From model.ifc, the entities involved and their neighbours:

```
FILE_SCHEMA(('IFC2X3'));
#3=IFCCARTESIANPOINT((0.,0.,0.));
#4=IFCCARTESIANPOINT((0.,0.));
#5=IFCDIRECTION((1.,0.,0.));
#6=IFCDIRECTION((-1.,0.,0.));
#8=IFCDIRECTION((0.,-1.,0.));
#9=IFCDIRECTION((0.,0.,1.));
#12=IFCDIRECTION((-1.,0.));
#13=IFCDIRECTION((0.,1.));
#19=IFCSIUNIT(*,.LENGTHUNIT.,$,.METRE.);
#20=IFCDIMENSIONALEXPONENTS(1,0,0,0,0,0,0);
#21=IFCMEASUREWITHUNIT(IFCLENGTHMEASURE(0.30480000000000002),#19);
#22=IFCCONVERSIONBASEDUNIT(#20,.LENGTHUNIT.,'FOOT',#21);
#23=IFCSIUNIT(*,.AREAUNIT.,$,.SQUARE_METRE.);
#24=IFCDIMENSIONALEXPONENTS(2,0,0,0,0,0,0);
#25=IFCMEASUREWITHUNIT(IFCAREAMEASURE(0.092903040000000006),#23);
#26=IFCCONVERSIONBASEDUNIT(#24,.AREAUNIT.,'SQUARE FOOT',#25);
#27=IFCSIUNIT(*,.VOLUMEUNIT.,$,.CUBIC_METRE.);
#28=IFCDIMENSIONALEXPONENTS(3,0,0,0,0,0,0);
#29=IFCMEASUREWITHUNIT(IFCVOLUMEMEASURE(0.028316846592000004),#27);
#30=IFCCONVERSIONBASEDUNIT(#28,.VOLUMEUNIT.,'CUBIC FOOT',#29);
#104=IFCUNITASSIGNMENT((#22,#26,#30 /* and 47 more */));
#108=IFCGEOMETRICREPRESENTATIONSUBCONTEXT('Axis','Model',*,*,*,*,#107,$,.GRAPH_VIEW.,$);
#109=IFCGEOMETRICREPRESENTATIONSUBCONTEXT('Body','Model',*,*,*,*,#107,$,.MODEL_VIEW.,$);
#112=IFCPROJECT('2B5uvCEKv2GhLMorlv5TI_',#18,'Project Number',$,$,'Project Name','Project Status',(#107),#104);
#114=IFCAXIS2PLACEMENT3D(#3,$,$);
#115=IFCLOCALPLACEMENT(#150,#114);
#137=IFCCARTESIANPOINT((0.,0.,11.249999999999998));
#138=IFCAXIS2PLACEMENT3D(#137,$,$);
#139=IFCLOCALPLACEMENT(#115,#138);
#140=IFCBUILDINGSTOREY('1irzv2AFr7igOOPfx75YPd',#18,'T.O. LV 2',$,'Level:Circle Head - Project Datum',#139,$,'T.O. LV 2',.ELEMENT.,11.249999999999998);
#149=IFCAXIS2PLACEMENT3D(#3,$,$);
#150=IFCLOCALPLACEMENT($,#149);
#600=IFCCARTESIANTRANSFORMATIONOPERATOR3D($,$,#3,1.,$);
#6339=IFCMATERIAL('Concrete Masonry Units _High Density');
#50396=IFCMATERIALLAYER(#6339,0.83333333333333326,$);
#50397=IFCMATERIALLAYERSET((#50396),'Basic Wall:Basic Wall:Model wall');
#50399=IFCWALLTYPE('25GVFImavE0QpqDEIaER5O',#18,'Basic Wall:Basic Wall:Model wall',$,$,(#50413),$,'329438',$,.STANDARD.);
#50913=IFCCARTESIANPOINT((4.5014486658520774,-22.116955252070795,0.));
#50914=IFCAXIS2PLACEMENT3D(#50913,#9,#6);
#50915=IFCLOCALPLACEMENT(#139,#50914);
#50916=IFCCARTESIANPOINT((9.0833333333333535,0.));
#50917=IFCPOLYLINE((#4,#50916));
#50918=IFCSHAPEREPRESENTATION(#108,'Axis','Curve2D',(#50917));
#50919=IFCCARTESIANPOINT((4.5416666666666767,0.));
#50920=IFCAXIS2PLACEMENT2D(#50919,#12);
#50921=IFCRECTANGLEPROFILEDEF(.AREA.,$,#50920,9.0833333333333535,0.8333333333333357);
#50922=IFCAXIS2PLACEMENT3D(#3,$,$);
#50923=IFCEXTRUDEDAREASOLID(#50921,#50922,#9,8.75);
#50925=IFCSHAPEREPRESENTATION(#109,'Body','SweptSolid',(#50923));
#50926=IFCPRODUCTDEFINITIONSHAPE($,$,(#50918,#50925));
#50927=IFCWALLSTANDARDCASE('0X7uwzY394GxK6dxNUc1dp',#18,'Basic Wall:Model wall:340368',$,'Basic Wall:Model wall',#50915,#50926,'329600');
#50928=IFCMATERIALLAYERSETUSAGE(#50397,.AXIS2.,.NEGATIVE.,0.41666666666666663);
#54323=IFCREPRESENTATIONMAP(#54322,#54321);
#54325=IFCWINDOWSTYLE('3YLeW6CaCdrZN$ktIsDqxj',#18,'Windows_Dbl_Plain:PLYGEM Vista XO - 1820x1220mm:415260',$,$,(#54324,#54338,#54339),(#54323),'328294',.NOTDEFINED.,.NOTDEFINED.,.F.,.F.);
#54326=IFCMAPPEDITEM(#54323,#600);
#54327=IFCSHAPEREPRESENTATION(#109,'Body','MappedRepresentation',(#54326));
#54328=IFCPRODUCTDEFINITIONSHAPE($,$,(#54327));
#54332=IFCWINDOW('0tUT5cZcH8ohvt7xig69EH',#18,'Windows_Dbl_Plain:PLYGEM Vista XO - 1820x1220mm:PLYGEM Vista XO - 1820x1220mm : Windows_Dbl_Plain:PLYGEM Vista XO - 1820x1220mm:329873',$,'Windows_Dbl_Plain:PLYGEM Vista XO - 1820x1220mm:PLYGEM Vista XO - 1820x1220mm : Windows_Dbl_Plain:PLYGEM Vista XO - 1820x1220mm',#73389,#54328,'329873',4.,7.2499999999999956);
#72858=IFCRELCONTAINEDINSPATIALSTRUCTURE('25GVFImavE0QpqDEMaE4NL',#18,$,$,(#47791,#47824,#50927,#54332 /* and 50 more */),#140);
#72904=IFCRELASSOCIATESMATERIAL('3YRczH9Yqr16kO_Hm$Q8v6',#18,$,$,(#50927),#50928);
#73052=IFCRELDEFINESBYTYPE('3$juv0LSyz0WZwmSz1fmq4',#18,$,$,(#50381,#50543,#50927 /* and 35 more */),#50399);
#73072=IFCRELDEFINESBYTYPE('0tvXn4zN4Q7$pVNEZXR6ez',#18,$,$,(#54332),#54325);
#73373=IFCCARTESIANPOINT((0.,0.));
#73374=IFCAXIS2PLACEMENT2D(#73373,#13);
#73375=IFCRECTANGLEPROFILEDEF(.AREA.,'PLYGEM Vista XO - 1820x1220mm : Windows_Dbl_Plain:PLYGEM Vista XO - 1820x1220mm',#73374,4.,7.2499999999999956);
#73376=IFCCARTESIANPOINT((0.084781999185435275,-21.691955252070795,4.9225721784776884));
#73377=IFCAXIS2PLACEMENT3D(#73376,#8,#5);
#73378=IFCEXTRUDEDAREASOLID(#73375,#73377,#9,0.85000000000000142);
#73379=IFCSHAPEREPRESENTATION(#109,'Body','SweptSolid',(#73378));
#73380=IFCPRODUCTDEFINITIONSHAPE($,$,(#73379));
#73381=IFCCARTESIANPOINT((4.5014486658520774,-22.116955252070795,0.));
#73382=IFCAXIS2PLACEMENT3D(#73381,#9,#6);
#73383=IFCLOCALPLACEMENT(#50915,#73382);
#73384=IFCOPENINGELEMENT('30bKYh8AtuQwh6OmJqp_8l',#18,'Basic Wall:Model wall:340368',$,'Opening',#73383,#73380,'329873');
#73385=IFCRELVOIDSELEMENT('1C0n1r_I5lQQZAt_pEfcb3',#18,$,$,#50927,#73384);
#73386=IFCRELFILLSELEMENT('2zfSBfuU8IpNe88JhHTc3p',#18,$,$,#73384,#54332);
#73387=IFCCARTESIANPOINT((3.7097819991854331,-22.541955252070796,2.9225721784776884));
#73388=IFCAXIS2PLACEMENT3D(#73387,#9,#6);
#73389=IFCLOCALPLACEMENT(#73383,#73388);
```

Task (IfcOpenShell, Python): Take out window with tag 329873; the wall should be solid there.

```python
import ifcopenshell
import ifcopenshell.api.feature
import ifcopenshell.api.root
import ifcopenshell.geom
import ifcopenshell.util.shape

model = ifcopenshell.open("model.ifc")
settings = ifcopenshell.geom.settings()


def volume(element):
    """Net volume in cubic metres, openings subtracted."""
    shape = ifcopenshell.geom.create_shape(settings, element)
    return ifcopenshell.util.shape.get_volume(shape.geometry)


window = model.by_guid("0tUT5cZcH8ohvt7xig69EH")
opening = window.FillsVoids[0].RelatingOpeningElement
wall = opening.VoidsElements[0].RelatingBuildingElement
before = volume(wall)

ifcopenshell.api.root.remove_product(model, product=window)
ifcopenshell.api.feature.remove_feature(model, feature=opening)

after = volume(wall)

print(f"wall volume {before:.3f} -> {after:.3f} m3")

model.write("model_updated.ifc")
```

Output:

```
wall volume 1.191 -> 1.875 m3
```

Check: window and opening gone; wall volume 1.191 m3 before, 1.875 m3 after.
